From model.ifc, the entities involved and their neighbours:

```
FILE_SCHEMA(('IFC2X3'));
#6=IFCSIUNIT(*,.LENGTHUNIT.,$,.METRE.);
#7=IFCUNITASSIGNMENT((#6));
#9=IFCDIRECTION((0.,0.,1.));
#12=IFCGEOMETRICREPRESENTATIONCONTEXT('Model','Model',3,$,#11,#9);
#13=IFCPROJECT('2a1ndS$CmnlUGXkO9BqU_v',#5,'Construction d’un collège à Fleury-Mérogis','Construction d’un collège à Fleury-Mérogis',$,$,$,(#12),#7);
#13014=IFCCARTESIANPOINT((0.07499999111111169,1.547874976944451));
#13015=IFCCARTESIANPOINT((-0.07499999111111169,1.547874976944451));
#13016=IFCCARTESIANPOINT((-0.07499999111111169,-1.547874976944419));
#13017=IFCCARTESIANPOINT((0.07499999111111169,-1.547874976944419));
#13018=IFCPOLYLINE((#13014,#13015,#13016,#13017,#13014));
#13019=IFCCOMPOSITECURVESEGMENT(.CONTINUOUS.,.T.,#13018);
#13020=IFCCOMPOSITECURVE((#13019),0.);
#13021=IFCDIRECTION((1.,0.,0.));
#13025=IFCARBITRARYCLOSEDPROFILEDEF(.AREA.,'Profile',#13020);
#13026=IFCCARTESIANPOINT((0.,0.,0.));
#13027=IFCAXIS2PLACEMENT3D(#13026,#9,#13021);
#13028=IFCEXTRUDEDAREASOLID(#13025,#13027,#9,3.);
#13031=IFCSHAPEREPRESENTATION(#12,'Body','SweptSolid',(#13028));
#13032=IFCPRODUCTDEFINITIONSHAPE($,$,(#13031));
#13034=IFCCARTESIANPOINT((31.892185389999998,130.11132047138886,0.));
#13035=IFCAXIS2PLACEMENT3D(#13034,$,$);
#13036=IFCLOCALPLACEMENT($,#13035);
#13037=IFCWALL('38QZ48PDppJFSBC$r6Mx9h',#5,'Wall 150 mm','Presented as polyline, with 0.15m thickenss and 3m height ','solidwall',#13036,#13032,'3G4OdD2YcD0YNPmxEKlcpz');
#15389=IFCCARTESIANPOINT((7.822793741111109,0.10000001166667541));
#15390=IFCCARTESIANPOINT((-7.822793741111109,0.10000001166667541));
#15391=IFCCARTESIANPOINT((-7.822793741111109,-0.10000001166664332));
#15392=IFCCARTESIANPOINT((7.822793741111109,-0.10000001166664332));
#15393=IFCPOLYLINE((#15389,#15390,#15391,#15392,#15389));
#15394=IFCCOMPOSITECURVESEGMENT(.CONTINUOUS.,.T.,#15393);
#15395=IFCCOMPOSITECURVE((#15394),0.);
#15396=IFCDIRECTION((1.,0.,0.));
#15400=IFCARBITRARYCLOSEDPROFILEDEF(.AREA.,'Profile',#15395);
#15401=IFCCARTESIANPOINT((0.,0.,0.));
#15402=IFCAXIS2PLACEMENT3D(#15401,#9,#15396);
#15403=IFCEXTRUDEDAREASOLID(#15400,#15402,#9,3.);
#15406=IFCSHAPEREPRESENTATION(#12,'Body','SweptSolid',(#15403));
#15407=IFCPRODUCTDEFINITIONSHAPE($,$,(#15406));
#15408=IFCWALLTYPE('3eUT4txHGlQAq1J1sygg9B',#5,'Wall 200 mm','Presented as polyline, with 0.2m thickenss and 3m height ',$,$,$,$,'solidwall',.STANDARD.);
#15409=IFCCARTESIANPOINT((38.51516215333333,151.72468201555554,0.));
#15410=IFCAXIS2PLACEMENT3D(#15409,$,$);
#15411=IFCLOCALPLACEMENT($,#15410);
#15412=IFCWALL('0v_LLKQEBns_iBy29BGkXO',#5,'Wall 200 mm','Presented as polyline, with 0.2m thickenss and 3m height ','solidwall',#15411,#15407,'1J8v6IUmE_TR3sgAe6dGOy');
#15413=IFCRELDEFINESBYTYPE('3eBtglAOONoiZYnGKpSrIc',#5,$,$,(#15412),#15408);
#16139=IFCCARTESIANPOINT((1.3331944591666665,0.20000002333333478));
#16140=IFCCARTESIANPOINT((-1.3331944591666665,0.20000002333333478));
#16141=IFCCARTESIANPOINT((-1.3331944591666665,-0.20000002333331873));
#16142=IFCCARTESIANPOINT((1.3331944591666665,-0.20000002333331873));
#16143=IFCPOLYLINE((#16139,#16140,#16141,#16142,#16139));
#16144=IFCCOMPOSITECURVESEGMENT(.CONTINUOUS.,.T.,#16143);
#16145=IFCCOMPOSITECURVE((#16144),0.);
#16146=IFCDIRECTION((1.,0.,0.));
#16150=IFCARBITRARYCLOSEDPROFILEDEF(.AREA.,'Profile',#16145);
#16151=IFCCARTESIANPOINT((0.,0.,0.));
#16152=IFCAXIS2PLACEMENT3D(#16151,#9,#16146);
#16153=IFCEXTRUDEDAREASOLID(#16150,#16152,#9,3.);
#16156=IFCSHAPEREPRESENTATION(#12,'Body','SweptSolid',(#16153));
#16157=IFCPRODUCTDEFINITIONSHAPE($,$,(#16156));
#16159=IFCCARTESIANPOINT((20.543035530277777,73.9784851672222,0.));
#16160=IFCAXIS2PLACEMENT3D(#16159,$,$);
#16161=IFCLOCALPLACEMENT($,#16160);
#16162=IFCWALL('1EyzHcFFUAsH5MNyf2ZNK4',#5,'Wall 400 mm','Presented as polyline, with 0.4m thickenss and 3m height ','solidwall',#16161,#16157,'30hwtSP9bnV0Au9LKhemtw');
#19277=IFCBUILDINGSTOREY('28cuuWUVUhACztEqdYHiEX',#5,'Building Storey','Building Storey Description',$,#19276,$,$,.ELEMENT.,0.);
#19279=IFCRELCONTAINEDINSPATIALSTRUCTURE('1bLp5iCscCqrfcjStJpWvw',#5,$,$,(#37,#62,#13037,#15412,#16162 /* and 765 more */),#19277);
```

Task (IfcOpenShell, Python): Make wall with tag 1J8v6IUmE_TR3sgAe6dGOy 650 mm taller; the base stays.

```python
import ifcopenshell
import ifcopenshell.geom
import ifcopenshell.util.shape
import ifcopenshell.util.unit

model = ifcopenshell.open("model.ifc")
unit_scale = ifcopenshell.util.unit.calculate_unit_scale(model)
settings = ifcopenshell.geom.settings()


def volume(element):
    """Net volume in cubic metres, openings subtracted."""
    shape = ifcopenshell.geom.create_shape(settings, element)
    return ifcopenshell.util.shape.get_volume(shape.geometry)


wall = model.by_guid("0v_LLKQEBns_iBy29BGkXO")
before = volume(wall)

body = next(r for r in wall.Representation.Representations if r.RepresentationIdentifier == "Body")
solid = body.Items[0]
old_height = solid.Depth
solid.Depth += 0.65 / unit_scale
after = volume(wall)

print(f"height {old_height:g} -> {solid.Depth:g}, volume {before:.3f} -> {after:.3f} m3")

model.write("model-out.ifc")
```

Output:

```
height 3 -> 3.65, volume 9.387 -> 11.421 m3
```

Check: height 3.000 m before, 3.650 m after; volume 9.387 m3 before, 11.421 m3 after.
